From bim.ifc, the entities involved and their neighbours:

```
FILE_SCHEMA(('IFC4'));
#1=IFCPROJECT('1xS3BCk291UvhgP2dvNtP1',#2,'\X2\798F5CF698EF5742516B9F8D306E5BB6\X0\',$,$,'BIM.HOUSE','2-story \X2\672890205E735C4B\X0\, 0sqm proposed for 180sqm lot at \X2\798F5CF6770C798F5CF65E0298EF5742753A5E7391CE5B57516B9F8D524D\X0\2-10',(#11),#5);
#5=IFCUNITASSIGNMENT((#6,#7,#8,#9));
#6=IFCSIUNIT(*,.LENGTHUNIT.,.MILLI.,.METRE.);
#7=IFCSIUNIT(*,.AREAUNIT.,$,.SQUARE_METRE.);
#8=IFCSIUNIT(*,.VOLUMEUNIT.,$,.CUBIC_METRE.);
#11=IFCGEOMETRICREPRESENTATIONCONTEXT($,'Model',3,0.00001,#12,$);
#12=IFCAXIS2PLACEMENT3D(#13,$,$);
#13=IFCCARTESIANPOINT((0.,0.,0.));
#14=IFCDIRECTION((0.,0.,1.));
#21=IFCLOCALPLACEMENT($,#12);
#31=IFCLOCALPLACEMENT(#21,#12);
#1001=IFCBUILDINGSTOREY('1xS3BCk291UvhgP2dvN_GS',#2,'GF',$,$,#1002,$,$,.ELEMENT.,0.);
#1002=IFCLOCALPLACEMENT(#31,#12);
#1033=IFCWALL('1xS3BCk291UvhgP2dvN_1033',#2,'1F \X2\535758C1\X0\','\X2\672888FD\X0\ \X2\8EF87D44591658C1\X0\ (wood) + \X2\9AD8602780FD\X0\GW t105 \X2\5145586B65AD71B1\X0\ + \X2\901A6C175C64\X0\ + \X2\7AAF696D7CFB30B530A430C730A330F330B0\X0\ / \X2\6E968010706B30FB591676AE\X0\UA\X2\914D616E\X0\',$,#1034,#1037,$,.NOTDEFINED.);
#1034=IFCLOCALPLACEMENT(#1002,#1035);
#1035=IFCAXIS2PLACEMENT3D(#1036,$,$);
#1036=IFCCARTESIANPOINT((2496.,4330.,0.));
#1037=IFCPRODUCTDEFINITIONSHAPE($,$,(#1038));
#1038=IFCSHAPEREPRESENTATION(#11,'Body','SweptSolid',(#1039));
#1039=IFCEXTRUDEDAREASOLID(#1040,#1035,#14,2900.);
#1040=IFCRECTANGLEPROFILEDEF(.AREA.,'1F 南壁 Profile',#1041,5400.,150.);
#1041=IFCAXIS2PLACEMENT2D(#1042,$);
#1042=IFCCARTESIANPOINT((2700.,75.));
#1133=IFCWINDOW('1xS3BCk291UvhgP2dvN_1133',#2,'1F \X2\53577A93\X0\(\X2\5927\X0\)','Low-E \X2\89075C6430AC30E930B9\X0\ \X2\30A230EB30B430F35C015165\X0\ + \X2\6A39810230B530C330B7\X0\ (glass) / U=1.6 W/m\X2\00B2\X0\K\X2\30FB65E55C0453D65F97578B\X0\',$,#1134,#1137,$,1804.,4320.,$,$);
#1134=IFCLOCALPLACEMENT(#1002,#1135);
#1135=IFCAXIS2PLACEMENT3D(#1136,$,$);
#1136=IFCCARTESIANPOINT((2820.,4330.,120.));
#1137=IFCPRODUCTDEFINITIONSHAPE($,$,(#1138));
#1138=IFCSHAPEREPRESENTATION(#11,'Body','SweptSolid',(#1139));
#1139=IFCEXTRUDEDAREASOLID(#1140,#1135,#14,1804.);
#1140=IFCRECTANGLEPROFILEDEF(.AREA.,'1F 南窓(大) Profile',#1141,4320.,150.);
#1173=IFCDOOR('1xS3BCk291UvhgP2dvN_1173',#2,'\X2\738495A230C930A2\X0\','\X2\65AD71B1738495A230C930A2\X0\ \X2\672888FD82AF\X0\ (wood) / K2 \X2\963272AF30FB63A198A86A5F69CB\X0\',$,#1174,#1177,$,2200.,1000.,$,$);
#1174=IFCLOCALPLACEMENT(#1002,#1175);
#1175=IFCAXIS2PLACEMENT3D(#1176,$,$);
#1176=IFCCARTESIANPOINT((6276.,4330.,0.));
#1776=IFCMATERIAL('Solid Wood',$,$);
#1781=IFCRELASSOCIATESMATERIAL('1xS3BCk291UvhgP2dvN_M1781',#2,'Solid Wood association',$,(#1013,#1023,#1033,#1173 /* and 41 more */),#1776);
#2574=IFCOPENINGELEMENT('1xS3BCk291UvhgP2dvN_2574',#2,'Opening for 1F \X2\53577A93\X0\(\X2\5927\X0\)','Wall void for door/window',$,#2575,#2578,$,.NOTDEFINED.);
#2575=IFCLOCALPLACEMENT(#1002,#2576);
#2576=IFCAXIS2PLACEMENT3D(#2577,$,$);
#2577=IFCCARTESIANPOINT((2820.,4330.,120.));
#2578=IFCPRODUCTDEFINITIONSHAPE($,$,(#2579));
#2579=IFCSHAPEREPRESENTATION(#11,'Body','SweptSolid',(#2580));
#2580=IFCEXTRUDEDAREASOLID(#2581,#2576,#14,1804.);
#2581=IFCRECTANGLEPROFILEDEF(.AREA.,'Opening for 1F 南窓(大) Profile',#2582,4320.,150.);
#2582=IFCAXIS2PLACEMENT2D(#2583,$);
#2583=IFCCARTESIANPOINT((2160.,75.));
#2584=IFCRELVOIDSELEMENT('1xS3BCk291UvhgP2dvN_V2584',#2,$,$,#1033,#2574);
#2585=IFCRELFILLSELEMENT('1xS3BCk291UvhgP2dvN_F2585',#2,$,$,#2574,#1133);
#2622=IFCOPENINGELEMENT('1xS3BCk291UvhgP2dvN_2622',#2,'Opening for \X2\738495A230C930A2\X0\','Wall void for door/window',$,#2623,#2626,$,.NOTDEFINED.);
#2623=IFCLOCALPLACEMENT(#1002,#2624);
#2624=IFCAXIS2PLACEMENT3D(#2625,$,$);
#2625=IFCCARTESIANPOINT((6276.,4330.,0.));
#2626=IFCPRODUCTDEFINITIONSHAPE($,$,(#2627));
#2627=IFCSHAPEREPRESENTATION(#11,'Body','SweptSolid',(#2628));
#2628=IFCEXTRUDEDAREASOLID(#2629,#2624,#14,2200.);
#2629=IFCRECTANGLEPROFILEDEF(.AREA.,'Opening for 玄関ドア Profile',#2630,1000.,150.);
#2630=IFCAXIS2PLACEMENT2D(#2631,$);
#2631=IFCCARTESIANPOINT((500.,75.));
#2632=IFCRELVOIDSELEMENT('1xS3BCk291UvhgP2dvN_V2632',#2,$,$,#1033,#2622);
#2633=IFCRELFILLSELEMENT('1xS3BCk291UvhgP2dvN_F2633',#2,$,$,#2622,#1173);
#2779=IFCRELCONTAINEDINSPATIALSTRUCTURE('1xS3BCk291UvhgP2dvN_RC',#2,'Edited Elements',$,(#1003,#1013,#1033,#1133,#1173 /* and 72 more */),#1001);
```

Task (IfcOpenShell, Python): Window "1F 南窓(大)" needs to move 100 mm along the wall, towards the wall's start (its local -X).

```python
import ifcopenshell
import ifcopenshell.api.geometry
import ifcopenshell.util.placement

model = ifcopenshell.open("bim.ifc")

window = model.by_guid("1xS3BCk291UvhgP2dvN_1133")
opening = window.FillsVoids[0].RelatingOpeningElement
wall = opening.VoidsElements[0].RelatingBuildingElement

wall_matrix = ifcopenshell.util.placement.get_local_placement(wall.ObjectPlacement)
shift = wall_matrix[:3, 0] * -100.0
before = ifcopenshell.util.placement.get_local_placement(window.ObjectPlacement)[:3, 3].copy()

# The window is not placed relative to its opening, so move both.
for product in (opening, window):
    matrix = ifcopenshell.util.placement.get_local_placement(product.ObjectPlacement)
    matrix[:3, 3] += shift
    ifcopenshell.api.geometry.edit_object_placement(model, product=product, matrix=matrix, is_si=False)

after = ifcopenshell.util.placement.get_local_placement(window.ObjectPlacement)[:3, 3]
print("window moved by", (after - before).round(3) + 0.0)

model.write("bim-out.ifc")
```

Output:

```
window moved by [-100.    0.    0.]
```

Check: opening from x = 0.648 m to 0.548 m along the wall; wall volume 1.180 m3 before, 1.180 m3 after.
